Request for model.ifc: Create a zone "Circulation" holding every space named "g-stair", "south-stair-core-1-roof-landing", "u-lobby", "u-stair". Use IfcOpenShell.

First a look at what the model holds.

```python
import ifcopenshell

model = ifcopenshell.open("model.ifc")
print(model.schema)
seen = {}
for space in model.by_type("IfcSpace"):
    seen[space.LongName] = seen.get(space.LongName, 0) + 1
for name, count in sorted(seen.items(), key=str):
    print(count, "x", name)
print("zones:", [z.Name for z in model.by_type("IfcZone")][:20])
```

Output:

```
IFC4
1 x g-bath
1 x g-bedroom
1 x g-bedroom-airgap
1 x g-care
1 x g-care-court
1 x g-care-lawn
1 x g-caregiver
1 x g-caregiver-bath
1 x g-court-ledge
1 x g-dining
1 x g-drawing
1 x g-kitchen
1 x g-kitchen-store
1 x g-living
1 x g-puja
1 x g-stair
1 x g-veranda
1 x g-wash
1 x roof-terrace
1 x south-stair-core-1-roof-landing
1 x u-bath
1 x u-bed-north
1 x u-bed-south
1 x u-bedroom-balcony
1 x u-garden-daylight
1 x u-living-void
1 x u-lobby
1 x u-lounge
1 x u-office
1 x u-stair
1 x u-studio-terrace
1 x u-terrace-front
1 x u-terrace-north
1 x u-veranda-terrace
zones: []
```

```python
import ifcopenshell
import ifcopenshell.api.group
import ifcopenshell.api.root

model = ifcopenshell.open("model.ifc")

names = {"g-stair", "south-stair-core-1-roof-landing", "u-lobby", "u-stair"}
spaces = [s for s in model.by_type("IfcSpace") if s.LongName in names]

zone = ifcopenshell.api.root.create_entity(model, ifc_class="IfcZone", name="Circulation")
ifcopenshell.api.group.assign_group(model, products=spaces, group=zone)
print(len(spaces), "spaces in", zone.Name)

model.write("model_rev.ifc")
```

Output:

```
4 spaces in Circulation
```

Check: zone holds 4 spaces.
